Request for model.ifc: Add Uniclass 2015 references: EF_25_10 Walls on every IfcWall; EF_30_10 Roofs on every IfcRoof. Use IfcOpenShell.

First a look at what the model holds.

```python
import ifcopenshell

model = ifcopenshell.open("model.ifc")
print(model.schema)
print("classifications:", [c.Name for c in model.by_type("IfcClassification")])
for ifc_class in ("IfcDoor", "IfcRoof", "IfcStair", "IfcWall", "IfcWindow"):
    print(ifc_class, len(model.by_type(ifc_class)))
```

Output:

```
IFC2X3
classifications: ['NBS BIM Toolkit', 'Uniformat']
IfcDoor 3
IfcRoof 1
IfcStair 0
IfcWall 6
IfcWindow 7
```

```python
import ifcopenshell
import ifcopenshell.api.classification

model = ifcopenshell.open("model.ifc")

# IFC2X3 requires Source and Edition and has no link from the project to the system.
system = model.create_entity("IfcClassification", Source="NBS", Edition="2015", Name="Uniclass 2015")

codes = {
    "IfcWall": ("EF_25_10", "Walls"),
    "IfcRoof": ("EF_30_10", "Roofs"),
}
for ifc_class, (code, name) in codes.items():
    products = model.by_type(ifc_class)
    ifcopenshell.api.classification.add_reference(
        model, products=products, classification=system, identification=code, name=name
    )
    print(code, len(products))

model.write("model_rev.ifc")
```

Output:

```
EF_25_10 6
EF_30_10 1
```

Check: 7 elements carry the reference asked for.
